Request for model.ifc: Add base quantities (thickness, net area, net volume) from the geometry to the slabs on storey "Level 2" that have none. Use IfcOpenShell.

First a look at what the model holds.

```python
import ifcopenshell
import ifcopenshell.util.element
import ifcopenshell.util.unit

model = ifcopenshell.open("model.ifc")
print(model.schema)
for unit_type in ("LENGTHUNIT", "AREAUNIT", "VOLUMEUNIT"):
    print(unit_type, ifcopenshell.util.unit.calculate_unit_scale(model, unit_type))
storey = next(s for s in model.by_type("IfcBuildingStorey") if s.Name == "Level 2")
slabs = [e for e in ifcopenshell.util.element.get_decomposition(storey) if e.is_a("IfcSlab")]
for e in sorted(slabs, key=lambda e: e.id()):
    print(e.id(), e.is_a(), e.Name, list(ifcopenshell.util.element.get_psets(e, qtos_only=True)), sep=" | ")
```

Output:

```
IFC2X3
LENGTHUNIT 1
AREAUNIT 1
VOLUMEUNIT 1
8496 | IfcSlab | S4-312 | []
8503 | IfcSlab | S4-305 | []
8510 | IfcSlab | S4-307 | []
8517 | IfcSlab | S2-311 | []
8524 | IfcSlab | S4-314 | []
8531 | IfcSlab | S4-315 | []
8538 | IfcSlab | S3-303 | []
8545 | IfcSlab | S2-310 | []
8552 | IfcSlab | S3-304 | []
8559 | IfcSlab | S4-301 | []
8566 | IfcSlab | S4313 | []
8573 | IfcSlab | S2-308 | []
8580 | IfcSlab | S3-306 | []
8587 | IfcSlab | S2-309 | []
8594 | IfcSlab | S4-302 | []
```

```python
import ifcopenshell
import ifcopenshell.api.pset
import ifcopenshell.geom
import ifcopenshell.util.element
import ifcopenshell.util.shape
import ifcopenshell.util.unit

model = ifcopenshell.open("model.ifc")
unit_scale = ifcopenshell.util.unit.calculate_unit_scale(model)
area_scale = ifcopenshell.util.unit.calculate_unit_scale(model, "AREAUNIT")
volume_scale = ifcopenshell.util.unit.calculate_unit_scale(model, "VOLUMEUNIT")
settings = ifcopenshell.geom.settings()

storey = next(s for s in model.by_type("IfcBuildingStorey") if s.Name == "Level 2")
slabs = [e for e in ifcopenshell.util.element.get_decomposition(storey) if e.is_a("IfcSlab")]

for e in sorted(slabs, key=lambda e: e.id()):
    if ifcopenshell.util.element.get_psets(e, qtos_only=True, should_inherit=False):
        continue
    # Geometry comes back in metres, in the element's own axes.
    shape = ifcopenshell.geom.create_shape(settings, e)
    values = {
        "Width": ifcopenshell.util.shape.get_z(shape.geometry) / unit_scale,
        "NetArea": ifcopenshell.util.shape.get_footprint_area(shape.geometry) / area_scale,
        "NetVolume": ifcopenshell.util.shape.get_volume(shape.geometry) / volume_scale,
    }
    qto = ifcopenshell.api.pset.add_qto(model, product=e, name="BaseQuantities")
    ifcopenshell.api.pset.edit_qto(model, qto=qto, properties=values)
    print(e.id(), {k: round(v, 3) for k, v in values.items()})

model.write("model_v2.ifc")
```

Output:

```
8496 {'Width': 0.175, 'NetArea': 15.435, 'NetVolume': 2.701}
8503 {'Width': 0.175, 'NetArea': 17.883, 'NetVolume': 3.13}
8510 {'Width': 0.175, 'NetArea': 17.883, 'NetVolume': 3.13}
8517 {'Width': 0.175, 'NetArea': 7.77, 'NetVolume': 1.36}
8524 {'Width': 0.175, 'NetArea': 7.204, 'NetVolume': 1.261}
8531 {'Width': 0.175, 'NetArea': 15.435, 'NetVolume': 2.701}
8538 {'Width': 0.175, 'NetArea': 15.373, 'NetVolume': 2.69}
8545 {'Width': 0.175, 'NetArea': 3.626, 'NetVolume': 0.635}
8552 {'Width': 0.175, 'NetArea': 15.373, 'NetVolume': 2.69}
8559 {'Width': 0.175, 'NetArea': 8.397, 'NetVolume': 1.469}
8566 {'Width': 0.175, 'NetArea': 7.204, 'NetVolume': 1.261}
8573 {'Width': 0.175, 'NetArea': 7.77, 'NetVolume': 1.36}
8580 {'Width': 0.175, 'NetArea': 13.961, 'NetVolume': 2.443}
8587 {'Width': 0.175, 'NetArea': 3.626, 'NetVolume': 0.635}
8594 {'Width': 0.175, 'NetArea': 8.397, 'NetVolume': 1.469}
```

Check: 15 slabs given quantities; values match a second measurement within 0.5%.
